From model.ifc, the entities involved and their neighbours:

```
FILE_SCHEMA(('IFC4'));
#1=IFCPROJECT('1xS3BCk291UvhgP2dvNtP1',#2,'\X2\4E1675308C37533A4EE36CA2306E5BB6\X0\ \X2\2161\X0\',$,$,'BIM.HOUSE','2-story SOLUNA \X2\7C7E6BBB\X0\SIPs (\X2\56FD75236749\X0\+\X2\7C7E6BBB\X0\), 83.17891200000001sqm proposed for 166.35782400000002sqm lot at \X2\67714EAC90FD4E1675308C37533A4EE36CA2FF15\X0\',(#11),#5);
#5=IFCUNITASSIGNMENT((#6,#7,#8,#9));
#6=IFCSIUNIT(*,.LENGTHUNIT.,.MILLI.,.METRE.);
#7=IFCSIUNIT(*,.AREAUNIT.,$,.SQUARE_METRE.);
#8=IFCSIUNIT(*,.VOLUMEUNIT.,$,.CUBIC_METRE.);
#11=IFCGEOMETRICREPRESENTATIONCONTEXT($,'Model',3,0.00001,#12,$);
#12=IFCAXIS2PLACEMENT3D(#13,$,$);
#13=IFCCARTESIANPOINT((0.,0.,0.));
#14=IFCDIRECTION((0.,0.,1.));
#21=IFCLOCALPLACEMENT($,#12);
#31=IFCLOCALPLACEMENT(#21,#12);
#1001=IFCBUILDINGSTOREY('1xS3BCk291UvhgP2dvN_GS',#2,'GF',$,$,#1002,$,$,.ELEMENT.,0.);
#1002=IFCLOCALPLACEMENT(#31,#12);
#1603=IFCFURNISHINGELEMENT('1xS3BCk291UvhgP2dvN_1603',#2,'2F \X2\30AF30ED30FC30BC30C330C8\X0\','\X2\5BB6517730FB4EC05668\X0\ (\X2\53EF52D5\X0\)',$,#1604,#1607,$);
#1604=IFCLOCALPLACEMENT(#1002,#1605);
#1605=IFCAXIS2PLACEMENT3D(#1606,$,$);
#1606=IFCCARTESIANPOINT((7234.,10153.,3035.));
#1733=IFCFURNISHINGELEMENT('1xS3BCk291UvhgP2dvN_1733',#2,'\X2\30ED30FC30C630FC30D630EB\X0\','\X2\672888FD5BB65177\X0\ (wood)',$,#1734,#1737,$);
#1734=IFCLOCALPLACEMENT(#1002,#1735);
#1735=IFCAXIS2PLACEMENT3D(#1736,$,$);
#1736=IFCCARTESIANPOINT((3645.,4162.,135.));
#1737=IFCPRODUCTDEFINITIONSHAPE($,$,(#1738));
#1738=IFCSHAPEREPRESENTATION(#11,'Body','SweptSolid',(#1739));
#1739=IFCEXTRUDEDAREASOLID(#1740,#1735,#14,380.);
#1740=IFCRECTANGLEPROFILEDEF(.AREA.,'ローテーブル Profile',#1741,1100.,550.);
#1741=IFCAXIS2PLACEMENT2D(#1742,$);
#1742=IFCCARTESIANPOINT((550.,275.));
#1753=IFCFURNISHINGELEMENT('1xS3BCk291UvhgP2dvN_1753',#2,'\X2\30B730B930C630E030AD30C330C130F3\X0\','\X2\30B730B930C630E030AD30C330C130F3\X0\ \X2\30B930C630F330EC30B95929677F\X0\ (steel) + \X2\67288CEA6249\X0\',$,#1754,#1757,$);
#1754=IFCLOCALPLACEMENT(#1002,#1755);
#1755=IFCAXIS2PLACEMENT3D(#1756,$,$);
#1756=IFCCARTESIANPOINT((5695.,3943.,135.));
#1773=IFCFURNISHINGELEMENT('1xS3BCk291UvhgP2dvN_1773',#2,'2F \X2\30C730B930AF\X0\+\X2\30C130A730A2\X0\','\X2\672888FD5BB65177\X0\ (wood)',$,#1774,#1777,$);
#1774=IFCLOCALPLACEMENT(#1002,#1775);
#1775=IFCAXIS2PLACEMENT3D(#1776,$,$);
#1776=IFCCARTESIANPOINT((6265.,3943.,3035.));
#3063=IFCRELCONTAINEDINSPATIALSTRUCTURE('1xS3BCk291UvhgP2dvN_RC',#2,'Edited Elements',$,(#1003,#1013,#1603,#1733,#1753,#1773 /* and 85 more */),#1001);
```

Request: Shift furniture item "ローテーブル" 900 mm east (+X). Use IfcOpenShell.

```python
import ifcopenshell
import ifcopenshell.api.geometry
import ifcopenshell.util.placement
import ifcopenshell.util.unit

model = ifcopenshell.open("model.ifc")
unit_scale = ifcopenshell.util.unit.calculate_unit_scale(model)

item = model.by_guid("1xS3BCk291UvhgP2dvN_1733")
matrix = ifcopenshell.util.placement.get_local_placement(item.ObjectPlacement)
matrix[0, 3] += 0.9 / unit_scale
ifcopenshell.api.geometry.edit_object_placement(model, product=item, matrix=matrix, is_si=False)

print(ifcopenshell.util.placement.get_local_placement(item.ObjectPlacement).round(3) + 0.0)

model.write("model-out.ifc")
```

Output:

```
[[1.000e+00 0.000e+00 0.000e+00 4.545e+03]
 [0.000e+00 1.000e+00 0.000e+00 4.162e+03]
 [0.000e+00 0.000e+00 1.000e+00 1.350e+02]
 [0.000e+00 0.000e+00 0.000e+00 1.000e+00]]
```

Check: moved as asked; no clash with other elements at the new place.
